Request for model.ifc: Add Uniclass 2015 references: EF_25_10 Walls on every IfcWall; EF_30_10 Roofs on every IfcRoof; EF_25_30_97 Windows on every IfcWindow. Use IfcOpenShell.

First a look at what the model holds.

```python
import ifcopenshell

model = ifcopenshell.open("model.ifc")
print(model.schema)
print("classifications:", [c.Name for c in model.by_type("IfcClassification")])
for ifc_class in ("IfcDoor", "IfcRoof", "IfcStair", "IfcWall", "IfcWindow"):
    print(ifc_class, len(model.by_type(ifc_class)))
```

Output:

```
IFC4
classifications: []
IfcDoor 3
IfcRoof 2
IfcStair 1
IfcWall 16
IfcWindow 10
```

```python
import ifcopenshell
import ifcopenshell.api.classification

model = ifcopenshell.open("model.ifc")

system = ifcopenshell.api.classification.add_classification(model, classification="Uniclass 2015")

codes = {
    "IfcWall": ("EF_25_10", "Walls"),
    "IfcRoof": ("EF_30_10", "Roofs"),
    "IfcWindow": ("EF_25_30_97", "Windows"),
}
for ifc_class, (code, name) in codes.items():
    products = model.by_type(ifc_class)
    ifcopenshell.api.classification.add_reference(
        model, products=products, classification=system, identification=code, name=name
    )
    print(code, len(products))

model.write("model_v2.ifc")
```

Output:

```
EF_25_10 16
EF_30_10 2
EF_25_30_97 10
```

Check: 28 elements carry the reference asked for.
